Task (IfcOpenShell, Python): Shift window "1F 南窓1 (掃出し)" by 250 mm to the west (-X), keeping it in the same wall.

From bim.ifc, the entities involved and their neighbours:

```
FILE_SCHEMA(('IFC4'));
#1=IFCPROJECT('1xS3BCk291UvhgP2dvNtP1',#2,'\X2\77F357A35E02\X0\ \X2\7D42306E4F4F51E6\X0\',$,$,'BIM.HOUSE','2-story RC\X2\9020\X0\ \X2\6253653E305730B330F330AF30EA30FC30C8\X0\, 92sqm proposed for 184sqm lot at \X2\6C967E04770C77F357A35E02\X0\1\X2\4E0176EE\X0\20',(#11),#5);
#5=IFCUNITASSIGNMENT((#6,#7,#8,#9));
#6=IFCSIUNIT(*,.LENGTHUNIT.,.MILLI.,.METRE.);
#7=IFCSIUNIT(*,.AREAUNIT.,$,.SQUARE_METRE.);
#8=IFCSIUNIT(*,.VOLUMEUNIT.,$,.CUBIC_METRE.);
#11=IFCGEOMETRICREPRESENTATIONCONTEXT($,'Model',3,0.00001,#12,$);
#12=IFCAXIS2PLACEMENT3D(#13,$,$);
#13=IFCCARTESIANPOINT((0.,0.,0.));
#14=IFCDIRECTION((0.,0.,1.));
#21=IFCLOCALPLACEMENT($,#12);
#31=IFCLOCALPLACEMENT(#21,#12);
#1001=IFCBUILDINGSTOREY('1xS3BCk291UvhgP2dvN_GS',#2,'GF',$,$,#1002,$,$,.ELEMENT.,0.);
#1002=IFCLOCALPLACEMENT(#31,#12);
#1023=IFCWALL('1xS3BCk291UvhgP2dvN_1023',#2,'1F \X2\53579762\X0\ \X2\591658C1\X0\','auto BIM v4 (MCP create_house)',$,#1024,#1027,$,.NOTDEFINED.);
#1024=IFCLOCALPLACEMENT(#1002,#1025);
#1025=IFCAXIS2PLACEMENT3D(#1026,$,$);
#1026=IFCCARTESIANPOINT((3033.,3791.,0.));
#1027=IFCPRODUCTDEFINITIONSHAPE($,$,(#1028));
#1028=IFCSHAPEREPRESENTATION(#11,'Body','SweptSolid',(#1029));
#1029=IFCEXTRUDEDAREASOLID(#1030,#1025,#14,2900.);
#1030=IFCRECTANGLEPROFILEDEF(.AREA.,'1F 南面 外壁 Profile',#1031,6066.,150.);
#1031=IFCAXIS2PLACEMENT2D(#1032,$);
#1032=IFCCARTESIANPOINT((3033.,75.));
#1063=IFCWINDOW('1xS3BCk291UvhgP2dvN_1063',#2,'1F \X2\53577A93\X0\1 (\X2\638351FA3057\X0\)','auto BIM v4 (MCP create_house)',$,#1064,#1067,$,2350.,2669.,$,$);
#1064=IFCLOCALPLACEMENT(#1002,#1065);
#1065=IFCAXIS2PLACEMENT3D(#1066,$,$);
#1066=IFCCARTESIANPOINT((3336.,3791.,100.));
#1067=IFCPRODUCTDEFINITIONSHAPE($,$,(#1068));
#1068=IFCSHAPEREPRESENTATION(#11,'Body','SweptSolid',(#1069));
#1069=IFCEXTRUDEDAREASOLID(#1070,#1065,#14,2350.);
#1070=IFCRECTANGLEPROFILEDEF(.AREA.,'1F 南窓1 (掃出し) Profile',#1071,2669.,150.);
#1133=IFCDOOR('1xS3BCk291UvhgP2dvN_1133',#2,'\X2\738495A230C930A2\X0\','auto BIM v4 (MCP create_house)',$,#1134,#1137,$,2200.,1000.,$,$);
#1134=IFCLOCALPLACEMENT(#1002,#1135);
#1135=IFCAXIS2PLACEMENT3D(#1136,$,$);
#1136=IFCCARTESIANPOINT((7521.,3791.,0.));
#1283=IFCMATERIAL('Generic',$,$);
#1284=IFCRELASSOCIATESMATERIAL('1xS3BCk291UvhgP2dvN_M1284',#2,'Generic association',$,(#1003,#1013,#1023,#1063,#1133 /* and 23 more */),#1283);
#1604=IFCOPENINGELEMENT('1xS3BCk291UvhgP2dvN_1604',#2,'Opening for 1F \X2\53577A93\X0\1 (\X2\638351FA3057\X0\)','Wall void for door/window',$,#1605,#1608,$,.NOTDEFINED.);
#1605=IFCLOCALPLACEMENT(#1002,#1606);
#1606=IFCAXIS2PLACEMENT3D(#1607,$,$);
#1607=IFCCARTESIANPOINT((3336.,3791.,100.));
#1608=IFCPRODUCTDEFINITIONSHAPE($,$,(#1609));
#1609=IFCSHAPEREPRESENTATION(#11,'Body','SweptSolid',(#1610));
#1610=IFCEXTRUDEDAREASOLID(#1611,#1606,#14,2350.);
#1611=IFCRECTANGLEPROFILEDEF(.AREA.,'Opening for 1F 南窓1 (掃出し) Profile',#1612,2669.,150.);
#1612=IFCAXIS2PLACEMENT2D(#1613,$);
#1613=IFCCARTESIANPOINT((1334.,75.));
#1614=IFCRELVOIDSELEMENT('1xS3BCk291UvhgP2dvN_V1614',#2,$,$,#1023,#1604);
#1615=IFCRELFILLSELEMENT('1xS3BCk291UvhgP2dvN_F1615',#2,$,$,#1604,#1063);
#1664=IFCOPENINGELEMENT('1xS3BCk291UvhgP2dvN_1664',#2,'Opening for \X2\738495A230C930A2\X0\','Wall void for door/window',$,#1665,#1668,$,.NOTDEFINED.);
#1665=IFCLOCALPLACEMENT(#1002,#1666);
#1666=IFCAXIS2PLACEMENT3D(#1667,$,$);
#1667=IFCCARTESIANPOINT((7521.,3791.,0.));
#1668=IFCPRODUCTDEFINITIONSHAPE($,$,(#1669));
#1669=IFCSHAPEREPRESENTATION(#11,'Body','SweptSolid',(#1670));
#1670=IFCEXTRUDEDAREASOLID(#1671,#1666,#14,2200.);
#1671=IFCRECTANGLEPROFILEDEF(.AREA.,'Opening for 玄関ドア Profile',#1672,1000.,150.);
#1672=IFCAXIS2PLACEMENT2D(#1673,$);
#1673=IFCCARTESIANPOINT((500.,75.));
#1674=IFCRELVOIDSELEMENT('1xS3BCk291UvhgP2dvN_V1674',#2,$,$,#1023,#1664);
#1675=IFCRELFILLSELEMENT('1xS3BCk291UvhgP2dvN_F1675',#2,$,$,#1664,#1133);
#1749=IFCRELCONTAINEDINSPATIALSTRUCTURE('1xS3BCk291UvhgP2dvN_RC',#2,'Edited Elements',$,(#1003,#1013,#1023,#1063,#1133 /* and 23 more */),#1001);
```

```python
import ifcopenshell
import ifcopenshell.api.geometry
import ifcopenshell.util.placement

model = ifcopenshell.open("bim.ifc")

window = model.by_guid("1xS3BCk291UvhgP2dvN_1063")
opening = window.FillsVoids[0].RelatingOpeningElement
wall = opening.VoidsElements[0].RelatingBuildingElement

wall_matrix = ifcopenshell.util.placement.get_local_placement(wall.ObjectPlacement)
shift = wall_matrix[:3, 0] * -250.0
before = ifcopenshell.util.placement.get_local_placement(window.ObjectPlacement)[:3, 3].copy()

# The window is not placed relative to its opening, so move both.
for product in (opening, window):
    matrix = ifcopenshell.util.placement.get_local_placement(product.ObjectPlacement)
    matrix[:3, 3] += shift
    ifcopenshell.api.geometry.edit_object_placement(model, product=product, matrix=matrix, is_si=False)

after = ifcopenshell.util.placement.get_local_placement(window.ObjectPlacement)[:3, 3]
print("window moved by", (after - before).round(3) + 0.0)

model.write("bim_v2.ifc")
```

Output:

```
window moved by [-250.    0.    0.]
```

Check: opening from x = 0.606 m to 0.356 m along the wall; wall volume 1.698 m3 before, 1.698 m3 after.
